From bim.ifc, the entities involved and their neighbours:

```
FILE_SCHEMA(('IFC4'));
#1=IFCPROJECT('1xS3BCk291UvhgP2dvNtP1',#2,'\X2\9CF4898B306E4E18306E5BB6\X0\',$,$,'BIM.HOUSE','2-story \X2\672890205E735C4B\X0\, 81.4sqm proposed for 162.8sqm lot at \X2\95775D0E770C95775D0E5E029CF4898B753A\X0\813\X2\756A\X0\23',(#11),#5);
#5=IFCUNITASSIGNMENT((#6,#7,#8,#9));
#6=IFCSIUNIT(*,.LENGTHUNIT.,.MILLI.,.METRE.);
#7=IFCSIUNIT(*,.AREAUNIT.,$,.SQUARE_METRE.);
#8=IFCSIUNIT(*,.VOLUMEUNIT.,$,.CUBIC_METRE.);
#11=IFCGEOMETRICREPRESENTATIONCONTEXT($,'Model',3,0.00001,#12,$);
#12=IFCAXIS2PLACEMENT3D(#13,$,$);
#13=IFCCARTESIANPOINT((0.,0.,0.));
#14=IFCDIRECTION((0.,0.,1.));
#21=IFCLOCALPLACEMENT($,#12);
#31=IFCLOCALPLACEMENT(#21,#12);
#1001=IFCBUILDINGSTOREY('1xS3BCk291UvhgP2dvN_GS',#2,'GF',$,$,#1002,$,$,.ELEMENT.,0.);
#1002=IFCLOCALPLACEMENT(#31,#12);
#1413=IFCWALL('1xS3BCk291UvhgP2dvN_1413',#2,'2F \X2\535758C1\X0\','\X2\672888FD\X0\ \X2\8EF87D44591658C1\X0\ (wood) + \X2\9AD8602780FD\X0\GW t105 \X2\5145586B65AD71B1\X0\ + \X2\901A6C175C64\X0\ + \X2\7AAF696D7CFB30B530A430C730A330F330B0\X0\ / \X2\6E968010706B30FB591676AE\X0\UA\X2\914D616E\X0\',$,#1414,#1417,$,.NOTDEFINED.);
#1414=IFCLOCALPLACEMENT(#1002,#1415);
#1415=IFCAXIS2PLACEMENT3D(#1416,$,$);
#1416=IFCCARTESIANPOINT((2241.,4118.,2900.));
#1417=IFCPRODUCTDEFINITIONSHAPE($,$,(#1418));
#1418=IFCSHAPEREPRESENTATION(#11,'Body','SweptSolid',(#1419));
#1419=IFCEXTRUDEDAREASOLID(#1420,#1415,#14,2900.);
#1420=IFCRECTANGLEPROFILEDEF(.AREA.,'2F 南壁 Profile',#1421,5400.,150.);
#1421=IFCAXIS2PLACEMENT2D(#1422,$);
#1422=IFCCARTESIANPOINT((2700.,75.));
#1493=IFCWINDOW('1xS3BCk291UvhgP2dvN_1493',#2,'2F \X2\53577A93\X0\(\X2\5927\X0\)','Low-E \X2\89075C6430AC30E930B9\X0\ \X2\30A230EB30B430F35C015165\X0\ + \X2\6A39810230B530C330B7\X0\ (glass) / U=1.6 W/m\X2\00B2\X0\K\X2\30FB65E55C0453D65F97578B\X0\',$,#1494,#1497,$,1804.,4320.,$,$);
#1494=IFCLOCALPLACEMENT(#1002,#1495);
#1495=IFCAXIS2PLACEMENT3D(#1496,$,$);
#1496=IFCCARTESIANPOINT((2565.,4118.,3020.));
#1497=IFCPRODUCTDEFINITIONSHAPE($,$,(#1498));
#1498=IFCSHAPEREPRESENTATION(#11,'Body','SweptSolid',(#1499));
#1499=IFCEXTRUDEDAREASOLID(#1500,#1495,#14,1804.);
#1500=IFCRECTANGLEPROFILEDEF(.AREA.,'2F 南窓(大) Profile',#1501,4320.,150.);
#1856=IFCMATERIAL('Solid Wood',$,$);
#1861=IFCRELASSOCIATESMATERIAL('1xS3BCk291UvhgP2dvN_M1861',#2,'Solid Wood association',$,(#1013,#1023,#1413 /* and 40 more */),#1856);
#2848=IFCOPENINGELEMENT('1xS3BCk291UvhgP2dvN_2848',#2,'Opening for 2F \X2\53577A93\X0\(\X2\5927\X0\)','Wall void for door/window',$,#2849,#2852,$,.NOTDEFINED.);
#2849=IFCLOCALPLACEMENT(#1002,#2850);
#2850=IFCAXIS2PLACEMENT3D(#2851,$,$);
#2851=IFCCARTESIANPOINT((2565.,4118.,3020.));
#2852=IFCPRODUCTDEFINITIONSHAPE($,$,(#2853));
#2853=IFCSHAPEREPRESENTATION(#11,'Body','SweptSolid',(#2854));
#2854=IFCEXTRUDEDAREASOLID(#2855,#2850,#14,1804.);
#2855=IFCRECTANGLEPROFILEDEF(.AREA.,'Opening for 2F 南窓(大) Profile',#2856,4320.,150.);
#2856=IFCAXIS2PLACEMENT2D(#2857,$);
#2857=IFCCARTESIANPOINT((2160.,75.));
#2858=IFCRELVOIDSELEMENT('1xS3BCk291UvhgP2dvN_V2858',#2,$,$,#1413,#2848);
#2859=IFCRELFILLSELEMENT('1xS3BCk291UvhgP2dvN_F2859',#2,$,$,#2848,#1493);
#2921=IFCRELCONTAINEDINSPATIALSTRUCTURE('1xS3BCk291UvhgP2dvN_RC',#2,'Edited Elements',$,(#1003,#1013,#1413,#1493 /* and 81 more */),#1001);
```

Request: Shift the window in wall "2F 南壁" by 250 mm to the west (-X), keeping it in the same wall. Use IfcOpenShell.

```python
import ifcopenshell
import ifcopenshell.api.geometry
import ifcopenshell.util.placement
import ifcopenshell.util.unit

model = ifcopenshell.open("bim.ifc")
unit_scale = ifcopenshell.util.unit.calculate_unit_scale(model)

window = model.by_guid("1xS3BCk291UvhgP2dvN_1493")
opening = window.FillsVoids[0].RelatingOpeningElement
wall = opening.VoidsElements[0].RelatingBuildingElement

wall_matrix = ifcopenshell.util.placement.get_local_placement(wall.ObjectPlacement)
shift = wall_matrix[:3, 0] * -0.25 / unit_scale
before = ifcopenshell.util.placement.get_local_placement(window.ObjectPlacement)[:3, 3].copy()

# The window is not placed relative to its opening, so move both.
for product in (opening, window):
    matrix = ifcopenshell.util.placement.get_local_placement(product.ObjectPlacement)
    matrix[:3, 3] += shift
    ifcopenshell.api.geometry.edit_object_placement(model, product=product, matrix=matrix, is_si=False)

after = ifcopenshell.util.placement.get_local_placement(window.ObjectPlacement)[:3, 3]
print("window moved by", (after - before).round(3) + 0.0)

model.write("bim-out.ifc")
```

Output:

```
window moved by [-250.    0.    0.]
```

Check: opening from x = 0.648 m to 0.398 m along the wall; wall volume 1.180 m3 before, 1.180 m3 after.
